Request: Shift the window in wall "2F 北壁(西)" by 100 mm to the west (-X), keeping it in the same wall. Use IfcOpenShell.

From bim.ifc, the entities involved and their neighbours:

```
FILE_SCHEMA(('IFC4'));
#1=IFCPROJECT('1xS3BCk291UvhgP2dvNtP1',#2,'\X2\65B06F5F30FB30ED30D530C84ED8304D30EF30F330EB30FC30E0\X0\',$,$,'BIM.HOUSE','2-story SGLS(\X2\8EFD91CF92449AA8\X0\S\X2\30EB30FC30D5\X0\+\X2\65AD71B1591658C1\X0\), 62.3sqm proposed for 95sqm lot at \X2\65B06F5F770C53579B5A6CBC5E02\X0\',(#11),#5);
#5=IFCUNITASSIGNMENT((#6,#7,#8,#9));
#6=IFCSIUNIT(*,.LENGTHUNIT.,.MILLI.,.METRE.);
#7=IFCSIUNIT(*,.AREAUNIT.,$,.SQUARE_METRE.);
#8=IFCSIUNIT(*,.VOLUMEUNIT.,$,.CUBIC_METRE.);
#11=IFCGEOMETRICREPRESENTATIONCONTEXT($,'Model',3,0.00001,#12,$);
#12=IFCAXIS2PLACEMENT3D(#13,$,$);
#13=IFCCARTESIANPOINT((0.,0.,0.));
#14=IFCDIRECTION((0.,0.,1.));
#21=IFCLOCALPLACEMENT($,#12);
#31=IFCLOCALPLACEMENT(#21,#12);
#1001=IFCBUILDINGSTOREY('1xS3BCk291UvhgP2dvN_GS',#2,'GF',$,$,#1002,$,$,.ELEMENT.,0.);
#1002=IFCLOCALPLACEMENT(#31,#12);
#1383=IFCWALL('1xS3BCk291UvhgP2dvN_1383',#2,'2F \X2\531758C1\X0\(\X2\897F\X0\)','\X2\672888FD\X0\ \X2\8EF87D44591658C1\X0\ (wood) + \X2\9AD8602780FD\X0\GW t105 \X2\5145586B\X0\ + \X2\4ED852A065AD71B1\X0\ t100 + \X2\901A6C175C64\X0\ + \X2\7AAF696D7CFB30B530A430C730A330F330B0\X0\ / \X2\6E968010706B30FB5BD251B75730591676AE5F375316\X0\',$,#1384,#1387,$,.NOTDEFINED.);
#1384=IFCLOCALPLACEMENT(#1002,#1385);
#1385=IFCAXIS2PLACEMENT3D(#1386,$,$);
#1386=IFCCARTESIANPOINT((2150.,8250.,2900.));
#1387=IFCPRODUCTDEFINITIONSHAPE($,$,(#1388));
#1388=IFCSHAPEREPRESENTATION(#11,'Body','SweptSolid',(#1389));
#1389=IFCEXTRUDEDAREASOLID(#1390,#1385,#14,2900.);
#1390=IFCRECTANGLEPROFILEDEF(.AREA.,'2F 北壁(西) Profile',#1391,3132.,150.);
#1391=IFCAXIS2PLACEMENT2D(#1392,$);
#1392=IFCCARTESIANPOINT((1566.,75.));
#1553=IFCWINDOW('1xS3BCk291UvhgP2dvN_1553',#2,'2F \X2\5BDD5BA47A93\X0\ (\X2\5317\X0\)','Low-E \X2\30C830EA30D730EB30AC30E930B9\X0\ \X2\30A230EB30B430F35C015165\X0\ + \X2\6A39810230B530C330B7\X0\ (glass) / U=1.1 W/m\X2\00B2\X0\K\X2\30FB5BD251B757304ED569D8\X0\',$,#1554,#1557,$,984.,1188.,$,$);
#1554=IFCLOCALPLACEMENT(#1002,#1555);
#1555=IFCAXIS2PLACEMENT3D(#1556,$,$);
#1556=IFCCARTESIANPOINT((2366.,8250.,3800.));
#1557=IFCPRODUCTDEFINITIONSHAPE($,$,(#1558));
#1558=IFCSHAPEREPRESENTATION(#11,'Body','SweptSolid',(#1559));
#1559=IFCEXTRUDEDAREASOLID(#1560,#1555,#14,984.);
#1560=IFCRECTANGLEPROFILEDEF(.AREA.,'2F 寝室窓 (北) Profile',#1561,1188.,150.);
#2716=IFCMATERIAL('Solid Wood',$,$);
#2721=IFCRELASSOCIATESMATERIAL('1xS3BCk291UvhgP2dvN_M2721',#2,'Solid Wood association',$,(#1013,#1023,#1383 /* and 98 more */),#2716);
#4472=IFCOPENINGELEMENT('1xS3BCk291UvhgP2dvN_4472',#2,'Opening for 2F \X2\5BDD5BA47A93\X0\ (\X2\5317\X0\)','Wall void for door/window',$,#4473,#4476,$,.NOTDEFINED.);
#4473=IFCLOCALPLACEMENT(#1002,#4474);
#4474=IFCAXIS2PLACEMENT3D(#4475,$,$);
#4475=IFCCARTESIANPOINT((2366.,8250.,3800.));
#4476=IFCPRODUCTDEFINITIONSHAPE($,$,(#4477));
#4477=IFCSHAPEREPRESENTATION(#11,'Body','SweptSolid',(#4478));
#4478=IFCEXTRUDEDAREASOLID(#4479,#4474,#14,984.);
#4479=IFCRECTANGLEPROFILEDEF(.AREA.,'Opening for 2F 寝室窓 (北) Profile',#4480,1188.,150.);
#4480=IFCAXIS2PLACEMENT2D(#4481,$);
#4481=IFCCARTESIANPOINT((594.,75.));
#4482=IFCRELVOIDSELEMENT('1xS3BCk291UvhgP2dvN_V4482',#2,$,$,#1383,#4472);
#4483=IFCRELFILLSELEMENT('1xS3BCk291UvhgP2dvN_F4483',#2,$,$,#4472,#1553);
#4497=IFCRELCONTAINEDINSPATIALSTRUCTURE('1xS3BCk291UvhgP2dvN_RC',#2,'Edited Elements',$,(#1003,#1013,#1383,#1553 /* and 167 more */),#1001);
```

```python
import ifcopenshell
import ifcopenshell.api.geometry
import ifcopenshell.util.placement

model = ifcopenshell.open("bim.ifc")

window = model.by_guid("1xS3BCk291UvhgP2dvN_1553")
opening = window.FillsVoids[0].RelatingOpeningElement
wall = opening.VoidsElements[0].RelatingBuildingElement

wall_matrix = ifcopenshell.util.placement.get_local_placement(wall.ObjectPlacement)
shift = wall_matrix[:3, 0] * -100.0
before = ifcopenshell.util.placement.get_local_placement(window.ObjectPlacement)[:3, 3].copy()

# The window is not placed relative to its opening, so move both.
for product in (opening, window):
    matrix = ifcopenshell.util.placement.get_local_placement(product.ObjectPlacement)
    matrix[:3, 3] += shift
    ifcopenshell.api.geometry.edit_object_placement(model, product=product, matrix=matrix, is_si=False)

after = ifcopenshell.util.placement.get_local_placement(window.ObjectPlacement)[:3, 3]
print("window moved by", (after - before).round(3) + 0.0)

model.write("bim_edited.ifc")
```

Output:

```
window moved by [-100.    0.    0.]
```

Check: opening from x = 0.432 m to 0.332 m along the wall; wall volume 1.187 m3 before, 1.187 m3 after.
